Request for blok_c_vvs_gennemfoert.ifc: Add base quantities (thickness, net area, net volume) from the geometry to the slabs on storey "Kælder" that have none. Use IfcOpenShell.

First a look at what the model holds.

```python
import ifcopenshell
import ifcopenshell.util.element
import ifcopenshell.util.unit

model = ifcopenshell.open("blok_c_vvs_gennemfoert.ifc")
print(model.schema)
for unit_type in ("LENGTHUNIT", "AREAUNIT", "VOLUMEUNIT"):
    print(unit_type, ifcopenshell.util.unit.calculate_unit_scale(model, unit_type))
storey = next(s for s in model.by_type("IfcBuildingStorey") if s.Name == "Kælder")
slabs = [e for e in ifcopenshell.util.element.get_decomposition(storey) if e.is_a("IfcSlab")]
for e in sorted(slabs, key=lambda e: e.id()):
    print(e.id(), e.is_a(), e.Name, list(ifcopenshell.util.element.get_psets(e, qtos_only=True)), sep=" | ")
```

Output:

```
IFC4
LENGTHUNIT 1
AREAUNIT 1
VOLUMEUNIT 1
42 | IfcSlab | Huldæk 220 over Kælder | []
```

```python
import ifcopenshell
import ifcopenshell.api.pset
import ifcopenshell.geom
import ifcopenshell.util.element
import ifcopenshell.util.shape
import ifcopenshell.util.unit

model = ifcopenshell.open("blok_c_vvs_gennemfoert.ifc")
unit_scale = ifcopenshell.util.unit.calculate_unit_scale(model)
area_scale = ifcopenshell.util.unit.calculate_unit_scale(model, "AREAUNIT")
volume_scale = ifcopenshell.util.unit.calculate_unit_scale(model, "VOLUMEUNIT")
settings = ifcopenshell.geom.settings()

storey = next(s for s in model.by_type("IfcBuildingStorey") if s.Name == "Kælder")
slabs = [e for e in ifcopenshell.util.element.get_decomposition(storey) if e.is_a("IfcSlab")]

for e in sorted(slabs, key=lambda e: e.id()):
    if ifcopenshell.util.element.get_psets(e, qtos_only=True, should_inherit=False):
        continue
    # Geometry comes back in metres, in the element's own axes.
    shape = ifcopenshell.geom.create_shape(settings, e)
    values = {
        "Width": ifcopenshell.util.shape.get_z(shape.geometry) / unit_scale,
        "NetArea": ifcopenshell.util.shape.get_footprint_area(shape.geometry) / area_scale,
        "NetVolume": ifcopenshell.util.shape.get_volume(shape.geometry) / volume_scale,
    }
    qto = ifcopenshell.api.pset.add_qto(model, product=e, name="Qto_SlabBaseQuantities")
    ifcopenshell.api.pset.edit_qto(model, qto=qto, properties=values)
    print(e.id(), {k: round(v, 3) for k, v in values.items()})

model.write("blok_c_vvs_gennemfoert_v2.ifc")
```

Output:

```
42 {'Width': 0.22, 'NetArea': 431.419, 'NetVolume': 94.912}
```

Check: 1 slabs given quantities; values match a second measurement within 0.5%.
